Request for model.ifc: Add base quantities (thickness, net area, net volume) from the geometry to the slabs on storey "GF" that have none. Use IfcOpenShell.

First a look at what the model holds.

```python
import ifcopenshell
import ifcopenshell.util.element
import ifcopenshell.util.unit

model = ifcopenshell.open("model.ifc")
print(model.schema)
for unit_type in ("LENGTHUNIT", "AREAUNIT", "VOLUMEUNIT"):
    print(unit_type, ifcopenshell.util.unit.calculate_unit_scale(model, unit_type))
storey = next(s for s in model.by_type("IfcBuildingStorey") if s.Name == "GF")
slabs = [e for e in ifcopenshell.util.element.get_decomposition(storey) if e.is_a("IfcSlab")]
for e in sorted(slabs, key=lambda e: e.id()):
    print(e.id(), e.is_a(), e.Name, list(ifcopenshell.util.element.get_psets(e, qtos_only=True)), sep=" | ")
```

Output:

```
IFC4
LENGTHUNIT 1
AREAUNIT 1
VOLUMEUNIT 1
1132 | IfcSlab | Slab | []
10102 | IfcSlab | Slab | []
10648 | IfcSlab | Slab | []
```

```python
import ifcopenshell
import ifcopenshell.api.pset
import ifcopenshell.geom
import ifcopenshell.util.element
import ifcopenshell.util.shape
import ifcopenshell.util.unit

model = ifcopenshell.open("model.ifc")
unit_scale = ifcopenshell.util.unit.calculate_unit_scale(model)
area_scale = ifcopenshell.util.unit.calculate_unit_scale(model, "AREAUNIT")
volume_scale = ifcopenshell.util.unit.calculate_unit_scale(model, "VOLUMEUNIT")
settings = ifcopenshell.geom.settings()

storey = next(s for s in model.by_type("IfcBuildingStorey") if s.Name == "GF")
slabs = [e for e in ifcopenshell.util.element.get_decomposition(storey) if e.is_a("IfcSlab")]

for e in sorted(slabs, key=lambda e: e.id()):
    if ifcopenshell.util.element.get_psets(e, qtos_only=True, should_inherit=False):
        continue
    # Geometry comes back in metres, in the element's own axes.
    shape = ifcopenshell.geom.create_shape(settings, e)
    values = {
        "Width": ifcopenshell.util.shape.get_z(shape.geometry) / unit_scale,
        "NetArea": ifcopenshell.util.shape.get_footprint_area(shape.geometry) / area_scale,
        "NetVolume": ifcopenshell.util.shape.get_volume(shape.geometry) / volume_scale,
    }
    qto = ifcopenshell.api.pset.add_qto(model, product=e, name="Qto_SlabBaseQuantities")
    ifcopenshell.api.pset.edit_qto(model, qto=qto, properties=values)
    print(e.id(), {k: round(v, 3) for k, v in values.items()})

model.write("model_updated.ifc")
```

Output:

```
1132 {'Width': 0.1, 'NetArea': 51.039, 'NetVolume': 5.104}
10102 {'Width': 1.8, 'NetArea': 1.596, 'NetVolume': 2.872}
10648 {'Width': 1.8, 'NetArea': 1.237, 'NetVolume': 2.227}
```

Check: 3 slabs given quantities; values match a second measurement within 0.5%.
